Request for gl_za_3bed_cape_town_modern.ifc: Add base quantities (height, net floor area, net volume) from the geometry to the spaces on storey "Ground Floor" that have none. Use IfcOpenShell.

First a look at what the model holds.

```python
import ifcopenshell
import ifcopenshell.util.element
import ifcopenshell.util.unit

model = ifcopenshell.open("gl_za_3bed_cape_town_modern.ifc")
print(model.schema)
for unit_type in ("LENGTHUNIT", "AREAUNIT", "VOLUMEUNIT"):
    print(unit_type, ifcopenshell.util.unit.calculate_unit_scale(model, unit_type))
storey = next(s for s in model.by_type("IfcBuildingStorey") if s.Name == "Ground Floor")
spaces = [e for e in ifcopenshell.util.element.get_decomposition(storey) if e.is_a("IfcSpace")]
for e in sorted(spaces, key=lambda e: e.id()):
    print(e.id(), e.is_a(), e.Name, list(ifcopenshell.util.element.get_psets(e, qtos_only=True)), sep=" | ")
```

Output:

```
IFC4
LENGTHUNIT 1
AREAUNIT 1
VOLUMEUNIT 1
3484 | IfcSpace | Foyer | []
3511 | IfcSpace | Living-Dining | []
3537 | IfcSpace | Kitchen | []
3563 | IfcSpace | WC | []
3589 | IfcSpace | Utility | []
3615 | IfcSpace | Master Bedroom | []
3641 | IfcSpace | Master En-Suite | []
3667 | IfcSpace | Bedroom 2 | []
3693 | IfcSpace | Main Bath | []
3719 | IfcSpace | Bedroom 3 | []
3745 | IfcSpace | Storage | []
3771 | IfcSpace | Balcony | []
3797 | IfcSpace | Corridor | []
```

```python
import ifcopenshell
import ifcopenshell.api.pset
import ifcopenshell.geom
import ifcopenshell.util.element
import ifcopenshell.util.shape
import ifcopenshell.util.unit

model = ifcopenshell.open("gl_za_3bed_cape_town_modern.ifc")
unit_scale = ifcopenshell.util.unit.calculate_unit_scale(model)
area_scale = ifcopenshell.util.unit.calculate_unit_scale(model, "AREAUNIT")
volume_scale = ifcopenshell.util.unit.calculate_unit_scale(model, "VOLUMEUNIT")
settings = ifcopenshell.geom.settings()

storey = next(s for s in model.by_type("IfcBuildingStorey") if s.Name == "Ground Floor")
spaces = [e for e in ifcopenshell.util.element.get_decomposition(storey) if e.is_a("IfcSpace")]

for e in sorted(spaces, key=lambda e: e.id()):
    if ifcopenshell.util.element.get_psets(e, qtos_only=True, should_inherit=False):
        continue
    # Geometry comes back in metres, in the element's own axes.
    shape = ifcopenshell.geom.create_shape(settings, e)
    values = {
        "Height": ifcopenshell.util.shape.get_z(shape.geometry) / unit_scale,
        "NetFloorArea": ifcopenshell.util.shape.get_footprint_area(shape.geometry) / area_scale,
        "NetVolume": ifcopenshell.util.shape.get_volume(shape.geometry) / volume_scale,
    }
    qto = ifcopenshell.api.pset.add_qto(model, product=e, name="Qto_SpaceBaseQuantities")
    ifcopenshell.api.pset.edit_qto(model, qto=qto, properties=values)
    print(e.id(), {k: round(v, 3) for k, v in values.items()})

model.write("gl_za_3bed_cape_town_modern_rev.ifc")
```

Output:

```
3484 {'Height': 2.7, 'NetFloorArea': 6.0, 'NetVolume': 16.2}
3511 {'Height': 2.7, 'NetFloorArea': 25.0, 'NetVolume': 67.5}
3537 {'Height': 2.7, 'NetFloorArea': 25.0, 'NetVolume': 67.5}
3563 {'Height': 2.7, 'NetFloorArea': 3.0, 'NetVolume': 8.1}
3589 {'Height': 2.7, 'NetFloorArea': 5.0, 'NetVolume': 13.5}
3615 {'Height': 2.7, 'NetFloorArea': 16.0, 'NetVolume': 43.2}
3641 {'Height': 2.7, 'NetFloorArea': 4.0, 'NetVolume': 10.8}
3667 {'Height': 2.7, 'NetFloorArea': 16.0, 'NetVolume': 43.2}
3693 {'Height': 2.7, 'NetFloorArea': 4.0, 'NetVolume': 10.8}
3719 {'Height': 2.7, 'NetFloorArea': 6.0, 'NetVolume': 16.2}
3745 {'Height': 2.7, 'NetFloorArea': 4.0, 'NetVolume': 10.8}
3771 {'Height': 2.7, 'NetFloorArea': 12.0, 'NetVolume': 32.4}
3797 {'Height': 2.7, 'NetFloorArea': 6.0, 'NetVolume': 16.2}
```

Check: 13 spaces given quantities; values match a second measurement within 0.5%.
